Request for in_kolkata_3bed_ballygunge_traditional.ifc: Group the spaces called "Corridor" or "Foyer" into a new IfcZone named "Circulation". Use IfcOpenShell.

First a look at what the model holds.

```python
import ifcopenshell

model = ifcopenshell.open("in_kolkata_3bed_ballygunge_traditional.ifc")
print(model.schema)
seen = {}
for space in model.by_type("IfcSpace"):
    seen[space.LongName] = seen.get(space.LongName, 0) + 1
for name, count in sorted(seen.items(), key=str):
    print(count, "x", name)
print("zones:", [z.Name for z in model.by_type("IfcZone")][:20])
```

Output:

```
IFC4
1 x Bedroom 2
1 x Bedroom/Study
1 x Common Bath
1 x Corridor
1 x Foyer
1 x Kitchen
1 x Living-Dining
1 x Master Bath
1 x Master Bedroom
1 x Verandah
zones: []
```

```python
import ifcopenshell
import ifcopenshell.api.group
import ifcopenshell.api.root

model = ifcopenshell.open("in_kolkata_3bed_ballygunge_traditional.ifc")

names = {"Corridor", "Foyer"}
spaces = [s for s in model.by_type("IfcSpace") if s.LongName in names]

zone = ifcopenshell.api.root.create_entity(model, ifc_class="IfcZone", name="Circulation")
ifcopenshell.api.group.assign_group(model, products=spaces, group=zone)
print(len(spaces), "spaces in", zone.Name)

model.write("in_kolkata_3bed_ballygunge_traditional-out.ifc")
```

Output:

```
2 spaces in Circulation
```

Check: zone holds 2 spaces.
